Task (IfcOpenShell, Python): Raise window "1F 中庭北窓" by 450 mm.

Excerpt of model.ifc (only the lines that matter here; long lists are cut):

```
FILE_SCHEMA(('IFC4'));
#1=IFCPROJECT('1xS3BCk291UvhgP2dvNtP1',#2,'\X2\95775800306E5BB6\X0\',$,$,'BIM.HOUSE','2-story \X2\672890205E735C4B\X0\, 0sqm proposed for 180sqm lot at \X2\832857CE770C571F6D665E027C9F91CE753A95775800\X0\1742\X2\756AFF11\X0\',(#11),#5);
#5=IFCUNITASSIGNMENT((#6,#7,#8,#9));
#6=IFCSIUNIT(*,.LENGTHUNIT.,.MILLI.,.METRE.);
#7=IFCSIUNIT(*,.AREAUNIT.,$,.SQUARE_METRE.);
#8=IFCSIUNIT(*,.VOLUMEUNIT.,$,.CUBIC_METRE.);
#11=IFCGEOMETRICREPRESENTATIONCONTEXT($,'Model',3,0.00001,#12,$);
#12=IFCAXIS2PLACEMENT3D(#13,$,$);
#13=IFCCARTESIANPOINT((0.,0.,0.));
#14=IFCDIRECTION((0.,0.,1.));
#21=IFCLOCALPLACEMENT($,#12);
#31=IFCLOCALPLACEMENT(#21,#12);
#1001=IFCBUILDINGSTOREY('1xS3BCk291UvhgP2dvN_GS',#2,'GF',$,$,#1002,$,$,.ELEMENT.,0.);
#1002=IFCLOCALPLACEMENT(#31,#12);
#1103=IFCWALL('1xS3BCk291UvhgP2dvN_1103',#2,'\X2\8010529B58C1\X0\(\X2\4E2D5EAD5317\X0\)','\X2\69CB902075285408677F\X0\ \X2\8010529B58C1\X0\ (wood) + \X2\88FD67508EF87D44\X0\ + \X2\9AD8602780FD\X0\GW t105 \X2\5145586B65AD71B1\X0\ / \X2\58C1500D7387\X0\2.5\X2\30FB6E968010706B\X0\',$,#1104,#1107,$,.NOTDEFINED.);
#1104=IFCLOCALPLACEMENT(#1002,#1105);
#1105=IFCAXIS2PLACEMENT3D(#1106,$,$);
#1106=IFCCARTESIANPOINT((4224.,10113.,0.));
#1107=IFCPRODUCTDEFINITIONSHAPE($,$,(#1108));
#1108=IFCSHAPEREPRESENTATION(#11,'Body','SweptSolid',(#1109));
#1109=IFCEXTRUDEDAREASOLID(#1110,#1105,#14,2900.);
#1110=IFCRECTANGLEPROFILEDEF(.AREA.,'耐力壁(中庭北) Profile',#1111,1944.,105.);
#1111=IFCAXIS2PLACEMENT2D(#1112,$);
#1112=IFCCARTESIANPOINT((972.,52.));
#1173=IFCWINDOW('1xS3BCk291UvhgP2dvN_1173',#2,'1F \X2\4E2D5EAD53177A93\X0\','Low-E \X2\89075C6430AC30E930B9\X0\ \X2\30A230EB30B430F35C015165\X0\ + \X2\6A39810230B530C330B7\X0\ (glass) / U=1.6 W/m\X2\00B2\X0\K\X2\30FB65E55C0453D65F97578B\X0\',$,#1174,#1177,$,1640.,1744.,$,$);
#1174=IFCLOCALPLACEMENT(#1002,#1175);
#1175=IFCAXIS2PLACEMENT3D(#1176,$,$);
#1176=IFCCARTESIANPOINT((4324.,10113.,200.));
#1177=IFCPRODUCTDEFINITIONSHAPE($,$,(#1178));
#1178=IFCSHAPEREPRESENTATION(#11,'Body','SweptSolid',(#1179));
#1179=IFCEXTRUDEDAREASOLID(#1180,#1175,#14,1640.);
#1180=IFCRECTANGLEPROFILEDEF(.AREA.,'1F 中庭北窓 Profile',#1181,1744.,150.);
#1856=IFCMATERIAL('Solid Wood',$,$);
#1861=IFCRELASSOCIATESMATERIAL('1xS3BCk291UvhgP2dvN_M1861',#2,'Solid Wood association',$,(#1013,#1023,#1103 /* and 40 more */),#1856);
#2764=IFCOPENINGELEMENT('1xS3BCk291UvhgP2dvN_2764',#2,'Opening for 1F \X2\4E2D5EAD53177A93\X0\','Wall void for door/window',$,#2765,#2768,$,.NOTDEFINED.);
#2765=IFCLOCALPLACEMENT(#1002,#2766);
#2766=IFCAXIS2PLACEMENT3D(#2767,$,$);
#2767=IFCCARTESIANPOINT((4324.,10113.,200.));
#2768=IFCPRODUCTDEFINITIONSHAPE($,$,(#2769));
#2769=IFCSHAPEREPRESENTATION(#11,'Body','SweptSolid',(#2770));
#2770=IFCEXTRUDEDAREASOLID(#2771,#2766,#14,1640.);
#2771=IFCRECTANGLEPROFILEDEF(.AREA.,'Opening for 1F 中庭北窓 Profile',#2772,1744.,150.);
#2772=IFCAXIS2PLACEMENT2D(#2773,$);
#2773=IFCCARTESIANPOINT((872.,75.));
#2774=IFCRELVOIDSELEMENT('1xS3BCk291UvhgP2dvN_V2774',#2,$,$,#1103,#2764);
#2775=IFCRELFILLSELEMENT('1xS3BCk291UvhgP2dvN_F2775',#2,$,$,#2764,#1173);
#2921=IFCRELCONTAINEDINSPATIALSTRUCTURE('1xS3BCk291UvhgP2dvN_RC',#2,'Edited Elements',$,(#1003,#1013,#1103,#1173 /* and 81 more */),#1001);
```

```python
import numpy as np
import ifcopenshell
import ifcopenshell.api.geometry
import ifcopenshell.util.placement
import ifcopenshell.util.unit

model = ifcopenshell.open("model.ifc")
unit_scale = ifcopenshell.util.unit.calculate_unit_scale(model)

window = model.by_guid("1xS3BCk291UvhgP2dvN_1173")
opening = window.FillsVoids[0].RelatingOpeningElement
dz = 450.0

shift = np.array([0.0, 0.0, dz])
# The window is not placed relative to its opening, so move both.
for product in (opening, window):
    matrix = ifcopenshell.util.placement.get_local_placement(product.ObjectPlacement)
    matrix[:3, 3] += shift
    ifcopenshell.api.geometry.edit_object_placement(model, product=product, matrix=matrix, is_si=False)

print(f"moved by {dz * unit_scale:+.3f} m")

model.write("model_updated.ifc")
```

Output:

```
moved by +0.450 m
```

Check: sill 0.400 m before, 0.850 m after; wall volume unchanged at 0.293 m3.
